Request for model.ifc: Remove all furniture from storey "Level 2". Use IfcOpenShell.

First a look at what the model holds.

```python
import ifcopenshell
import ifcopenshell.util.element

model = ifcopenshell.open("model.ifc")
print(model.schema)
storey = next(s for s in model.by_type("IfcBuildingStorey") if s.Name == "Level 2")
furniture = [e for e in ifcopenshell.util.element.get_decomposition(storey) if e.is_a("IfcFurnishingElement")]
seen = {}
for e in furniture:
    element_type = ifcopenshell.util.element.get_type(e)
    name = element_type.Name if element_type not in (None, e) else None
    seen[name] = seen.get(name, 0) + 1
for name, count in sorted(seen.items(), key=str):
    print(count, "x", name)
```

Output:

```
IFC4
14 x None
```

```python
import ifcopenshell
import ifcopenshell.api.root
import ifcopenshell.util.element

model = ifcopenshell.open("model.ifc")

storey = next(s for s in model.by_type("IfcBuildingStorey") if s.Name == "Level 2")
furniture = [e for e in ifcopenshell.util.element.get_decomposition(storey) if e.is_a("IfcFurnishingElement")]

for e in furniture:
    ifcopenshell.api.root.remove_product(model, product=e)
print(len(furniture), "removed")

model.write("model-out.ifc")
```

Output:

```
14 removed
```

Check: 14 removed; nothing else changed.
